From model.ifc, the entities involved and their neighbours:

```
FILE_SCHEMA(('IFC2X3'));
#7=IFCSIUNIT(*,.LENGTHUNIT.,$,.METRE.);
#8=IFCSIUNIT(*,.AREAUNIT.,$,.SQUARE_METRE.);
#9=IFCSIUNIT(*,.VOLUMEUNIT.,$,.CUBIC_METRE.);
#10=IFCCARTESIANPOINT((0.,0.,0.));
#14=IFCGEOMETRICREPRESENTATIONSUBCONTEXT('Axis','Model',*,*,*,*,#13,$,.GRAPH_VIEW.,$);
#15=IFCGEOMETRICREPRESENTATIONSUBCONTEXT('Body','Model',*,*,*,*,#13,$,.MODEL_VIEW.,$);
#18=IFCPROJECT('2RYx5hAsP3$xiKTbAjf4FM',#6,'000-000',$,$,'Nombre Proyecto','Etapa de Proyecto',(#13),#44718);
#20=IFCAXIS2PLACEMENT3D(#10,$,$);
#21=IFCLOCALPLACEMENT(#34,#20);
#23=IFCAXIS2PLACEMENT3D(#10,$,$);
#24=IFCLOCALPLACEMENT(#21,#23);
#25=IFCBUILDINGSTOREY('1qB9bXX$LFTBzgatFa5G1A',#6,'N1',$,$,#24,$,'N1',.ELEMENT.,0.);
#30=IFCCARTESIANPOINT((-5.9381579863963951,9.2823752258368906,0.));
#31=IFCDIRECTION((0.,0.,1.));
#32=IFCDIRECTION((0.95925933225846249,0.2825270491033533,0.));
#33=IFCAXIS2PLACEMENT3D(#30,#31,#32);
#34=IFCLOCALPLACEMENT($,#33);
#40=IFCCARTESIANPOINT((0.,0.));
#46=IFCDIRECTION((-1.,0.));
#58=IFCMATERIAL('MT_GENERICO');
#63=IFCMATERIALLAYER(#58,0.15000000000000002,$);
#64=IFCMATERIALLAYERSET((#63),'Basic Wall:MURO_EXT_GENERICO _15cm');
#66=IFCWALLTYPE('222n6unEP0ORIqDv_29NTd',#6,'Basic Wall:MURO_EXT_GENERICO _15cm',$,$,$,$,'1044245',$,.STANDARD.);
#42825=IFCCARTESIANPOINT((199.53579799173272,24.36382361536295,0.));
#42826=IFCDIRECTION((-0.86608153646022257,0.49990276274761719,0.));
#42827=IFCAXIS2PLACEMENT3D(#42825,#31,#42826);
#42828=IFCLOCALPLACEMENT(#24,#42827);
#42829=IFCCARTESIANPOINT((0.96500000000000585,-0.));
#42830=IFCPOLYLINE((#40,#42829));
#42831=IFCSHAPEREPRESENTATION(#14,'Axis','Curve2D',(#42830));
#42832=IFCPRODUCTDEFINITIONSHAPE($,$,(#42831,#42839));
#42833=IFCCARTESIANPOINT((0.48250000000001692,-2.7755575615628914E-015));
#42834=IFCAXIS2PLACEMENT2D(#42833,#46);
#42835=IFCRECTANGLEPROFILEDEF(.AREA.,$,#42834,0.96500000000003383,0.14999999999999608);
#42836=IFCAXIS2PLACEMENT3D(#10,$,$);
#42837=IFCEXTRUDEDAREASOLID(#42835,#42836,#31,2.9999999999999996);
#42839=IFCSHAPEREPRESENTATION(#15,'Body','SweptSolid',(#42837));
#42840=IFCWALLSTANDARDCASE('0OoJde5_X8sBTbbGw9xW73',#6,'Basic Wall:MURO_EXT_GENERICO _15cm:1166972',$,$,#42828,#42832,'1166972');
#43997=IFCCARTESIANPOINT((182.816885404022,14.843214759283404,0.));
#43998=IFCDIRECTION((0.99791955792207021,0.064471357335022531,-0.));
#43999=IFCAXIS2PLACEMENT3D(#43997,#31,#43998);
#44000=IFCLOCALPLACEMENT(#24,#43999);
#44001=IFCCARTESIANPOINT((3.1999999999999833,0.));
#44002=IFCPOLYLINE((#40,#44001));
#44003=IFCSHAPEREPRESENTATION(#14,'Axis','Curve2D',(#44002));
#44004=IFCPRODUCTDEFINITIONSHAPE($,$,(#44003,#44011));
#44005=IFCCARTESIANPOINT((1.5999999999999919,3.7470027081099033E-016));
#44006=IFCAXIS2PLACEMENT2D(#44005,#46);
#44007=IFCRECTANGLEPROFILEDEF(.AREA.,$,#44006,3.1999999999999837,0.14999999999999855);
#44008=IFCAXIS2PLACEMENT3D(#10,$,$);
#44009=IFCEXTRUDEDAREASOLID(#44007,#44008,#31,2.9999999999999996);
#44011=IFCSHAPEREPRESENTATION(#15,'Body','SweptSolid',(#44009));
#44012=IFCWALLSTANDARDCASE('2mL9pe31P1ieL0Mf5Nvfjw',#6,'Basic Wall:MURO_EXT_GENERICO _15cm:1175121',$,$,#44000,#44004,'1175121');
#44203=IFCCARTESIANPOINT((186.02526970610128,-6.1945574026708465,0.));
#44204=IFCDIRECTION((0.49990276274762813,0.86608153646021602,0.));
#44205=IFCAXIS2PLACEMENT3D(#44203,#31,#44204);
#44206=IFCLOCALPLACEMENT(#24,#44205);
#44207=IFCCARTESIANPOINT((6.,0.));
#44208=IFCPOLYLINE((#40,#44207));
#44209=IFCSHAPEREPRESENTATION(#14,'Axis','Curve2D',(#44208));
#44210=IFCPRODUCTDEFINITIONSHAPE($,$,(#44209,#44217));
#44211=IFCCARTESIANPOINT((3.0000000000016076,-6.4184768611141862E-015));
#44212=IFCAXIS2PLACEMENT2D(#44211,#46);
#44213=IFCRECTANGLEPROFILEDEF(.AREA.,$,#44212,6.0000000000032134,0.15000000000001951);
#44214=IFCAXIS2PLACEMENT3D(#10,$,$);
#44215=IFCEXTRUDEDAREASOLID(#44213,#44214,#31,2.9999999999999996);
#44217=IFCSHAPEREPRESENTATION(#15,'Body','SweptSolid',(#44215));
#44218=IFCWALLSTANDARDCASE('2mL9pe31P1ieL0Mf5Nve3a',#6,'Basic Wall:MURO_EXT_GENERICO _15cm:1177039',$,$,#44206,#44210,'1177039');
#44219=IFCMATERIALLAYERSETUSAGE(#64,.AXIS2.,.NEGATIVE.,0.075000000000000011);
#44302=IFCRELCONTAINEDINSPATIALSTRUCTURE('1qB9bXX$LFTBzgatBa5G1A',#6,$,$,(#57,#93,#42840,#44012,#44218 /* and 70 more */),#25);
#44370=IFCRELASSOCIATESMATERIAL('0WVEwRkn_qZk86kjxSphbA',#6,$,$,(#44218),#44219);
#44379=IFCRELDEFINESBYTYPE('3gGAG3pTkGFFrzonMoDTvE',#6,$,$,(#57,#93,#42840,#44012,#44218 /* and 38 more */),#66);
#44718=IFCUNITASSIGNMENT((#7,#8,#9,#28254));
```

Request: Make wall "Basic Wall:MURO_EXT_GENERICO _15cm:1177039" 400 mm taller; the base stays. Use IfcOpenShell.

```python
import ifcopenshell
import ifcopenshell.geom
import ifcopenshell.util.representation
import ifcopenshell.util.shape

model = ifcopenshell.open("model.ifc")
settings = ifcopenshell.geom.settings()


def volume(element):
    """Net volume in cubic metres, openings subtracted."""
    shape = ifcopenshell.geom.create_shape(settings, element)
    return ifcopenshell.util.shape.get_volume(shape.geometry)


wall = model.by_guid("2mL9pe31P1ieL0Mf5Nve3a")
before = volume(wall)

body = ifcopenshell.util.representation.get_representation(wall, "Model", "Body")
solid = body.Items[0]
old_height = solid.Depth
solid.Depth += 0.4
after = volume(wall)

print(f"height {old_height:g} -> {solid.Depth:g}, volume {before:.3f} -> {after:.3f} m3")

model.write("model_v2.ifc")
```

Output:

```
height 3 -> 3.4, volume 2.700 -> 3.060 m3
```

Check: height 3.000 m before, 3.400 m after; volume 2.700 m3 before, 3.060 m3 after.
